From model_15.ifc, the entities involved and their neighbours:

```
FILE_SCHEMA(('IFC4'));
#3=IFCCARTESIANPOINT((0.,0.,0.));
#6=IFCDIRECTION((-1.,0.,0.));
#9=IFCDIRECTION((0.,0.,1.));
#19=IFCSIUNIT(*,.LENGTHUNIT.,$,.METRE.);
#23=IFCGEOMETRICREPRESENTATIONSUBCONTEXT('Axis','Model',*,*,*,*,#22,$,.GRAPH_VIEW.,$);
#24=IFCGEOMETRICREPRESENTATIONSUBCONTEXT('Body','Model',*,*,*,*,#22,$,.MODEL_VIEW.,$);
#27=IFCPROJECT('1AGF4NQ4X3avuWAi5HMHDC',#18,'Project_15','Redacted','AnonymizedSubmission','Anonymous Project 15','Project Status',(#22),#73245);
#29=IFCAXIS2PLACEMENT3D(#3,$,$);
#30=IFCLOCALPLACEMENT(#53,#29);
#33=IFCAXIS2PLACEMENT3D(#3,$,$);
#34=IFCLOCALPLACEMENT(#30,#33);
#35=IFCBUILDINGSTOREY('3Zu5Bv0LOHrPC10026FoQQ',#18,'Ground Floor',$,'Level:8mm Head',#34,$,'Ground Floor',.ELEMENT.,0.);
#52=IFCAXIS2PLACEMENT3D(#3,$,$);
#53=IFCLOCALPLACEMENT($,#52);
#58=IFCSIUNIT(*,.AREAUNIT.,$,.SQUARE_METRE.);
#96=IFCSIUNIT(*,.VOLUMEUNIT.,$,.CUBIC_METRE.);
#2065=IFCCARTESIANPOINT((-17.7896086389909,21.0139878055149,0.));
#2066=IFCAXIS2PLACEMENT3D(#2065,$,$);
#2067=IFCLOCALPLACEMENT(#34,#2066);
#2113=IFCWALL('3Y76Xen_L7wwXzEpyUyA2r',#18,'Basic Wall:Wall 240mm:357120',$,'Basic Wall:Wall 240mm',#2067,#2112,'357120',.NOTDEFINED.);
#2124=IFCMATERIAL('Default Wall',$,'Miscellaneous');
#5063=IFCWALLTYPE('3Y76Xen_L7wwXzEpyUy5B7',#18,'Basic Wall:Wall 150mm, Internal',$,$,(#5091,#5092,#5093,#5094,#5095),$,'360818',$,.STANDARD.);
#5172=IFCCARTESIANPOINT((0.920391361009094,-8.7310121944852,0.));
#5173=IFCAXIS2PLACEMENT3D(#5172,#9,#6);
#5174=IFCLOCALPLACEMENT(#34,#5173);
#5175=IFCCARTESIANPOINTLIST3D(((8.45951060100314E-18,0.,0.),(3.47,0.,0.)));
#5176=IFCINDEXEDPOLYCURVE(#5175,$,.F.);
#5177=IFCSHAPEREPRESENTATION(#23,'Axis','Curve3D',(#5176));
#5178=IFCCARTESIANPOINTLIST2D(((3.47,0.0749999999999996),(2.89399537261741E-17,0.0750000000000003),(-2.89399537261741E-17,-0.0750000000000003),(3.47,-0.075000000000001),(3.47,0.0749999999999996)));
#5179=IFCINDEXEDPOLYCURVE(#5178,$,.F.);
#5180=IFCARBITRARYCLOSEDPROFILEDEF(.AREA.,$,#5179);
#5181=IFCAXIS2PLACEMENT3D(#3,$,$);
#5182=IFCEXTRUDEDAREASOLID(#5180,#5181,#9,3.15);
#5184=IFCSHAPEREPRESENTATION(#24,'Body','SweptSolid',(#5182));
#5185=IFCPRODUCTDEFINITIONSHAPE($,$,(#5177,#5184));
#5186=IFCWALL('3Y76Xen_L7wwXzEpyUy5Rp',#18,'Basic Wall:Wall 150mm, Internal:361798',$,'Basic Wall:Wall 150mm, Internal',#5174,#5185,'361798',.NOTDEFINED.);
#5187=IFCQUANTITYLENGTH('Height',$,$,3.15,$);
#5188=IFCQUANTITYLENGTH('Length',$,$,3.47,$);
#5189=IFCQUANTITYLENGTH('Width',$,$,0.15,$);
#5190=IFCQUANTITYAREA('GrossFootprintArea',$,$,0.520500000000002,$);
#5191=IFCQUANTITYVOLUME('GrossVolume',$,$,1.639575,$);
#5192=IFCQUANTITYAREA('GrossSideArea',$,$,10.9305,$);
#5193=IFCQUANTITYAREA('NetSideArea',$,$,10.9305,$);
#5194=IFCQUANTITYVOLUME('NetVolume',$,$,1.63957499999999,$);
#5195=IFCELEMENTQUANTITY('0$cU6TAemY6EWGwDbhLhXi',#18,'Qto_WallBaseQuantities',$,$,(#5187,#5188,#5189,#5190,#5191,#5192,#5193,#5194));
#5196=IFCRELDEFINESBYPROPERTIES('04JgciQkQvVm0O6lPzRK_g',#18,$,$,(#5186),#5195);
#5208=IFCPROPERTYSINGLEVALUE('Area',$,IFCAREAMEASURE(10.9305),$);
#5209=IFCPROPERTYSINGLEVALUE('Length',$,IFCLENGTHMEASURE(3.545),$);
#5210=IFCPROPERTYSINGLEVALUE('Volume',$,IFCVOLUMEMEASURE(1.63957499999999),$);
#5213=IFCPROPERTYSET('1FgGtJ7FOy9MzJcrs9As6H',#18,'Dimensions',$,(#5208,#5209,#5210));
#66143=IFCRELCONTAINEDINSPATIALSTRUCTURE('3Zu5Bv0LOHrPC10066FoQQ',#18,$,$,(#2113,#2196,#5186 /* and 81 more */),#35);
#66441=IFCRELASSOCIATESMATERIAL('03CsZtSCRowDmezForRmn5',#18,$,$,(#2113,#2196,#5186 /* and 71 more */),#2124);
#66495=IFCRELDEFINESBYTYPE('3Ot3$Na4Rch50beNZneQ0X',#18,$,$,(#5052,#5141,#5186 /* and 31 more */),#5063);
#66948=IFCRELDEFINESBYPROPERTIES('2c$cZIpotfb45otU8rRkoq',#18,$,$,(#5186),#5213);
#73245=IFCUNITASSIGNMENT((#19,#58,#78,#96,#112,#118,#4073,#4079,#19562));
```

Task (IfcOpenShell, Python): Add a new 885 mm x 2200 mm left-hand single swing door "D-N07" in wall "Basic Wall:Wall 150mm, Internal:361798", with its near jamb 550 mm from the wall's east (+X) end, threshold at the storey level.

```python
import numpy as np
import ifcopenshell
import ifcopenshell.api.feature
import ifcopenshell.api.geometry
import ifcopenshell.api.pset
import ifcopenshell.api.root
import ifcopenshell.api.spatial
import ifcopenshell.geom
import ifcopenshell.util.element
import ifcopenshell.util.placement
import ifcopenshell.util.representation
import ifcopenshell.util.shape
import ifcopenshell.util.unit

model = ifcopenshell.open("model_15.ifc")
unit_scale = ifcopenshell.util.unit.calculate_unit_scale(model)
area_scale = ifcopenshell.util.unit.calculate_unit_scale(model, "AREAUNIT")
volume_scale = ifcopenshell.util.unit.calculate_unit_scale(model, "VOLUMEUNIT")
settings = ifcopenshell.geom.settings()


def volume(element):
    """Net volume in cubic metres, openings subtracted."""
    shape = ifcopenshell.geom.create_shape(settings, element)
    return ifcopenshell.util.shape.get_volume(shape.geometry)


wall = model.by_guid("3Y76Xen_L7wwXzEpyUy5Rp")
storey = ifcopenshell.util.element.get_container(wall, ifc_class="IfcBuildingStorey")
context = ifcopenshell.util.representation.get_context(model, "Model", "Body", "MODEL_VIEW")
before = volume(wall)

width, height, from_end, sill = 0.885, 2.2, 0.55, 0.0  # metres

# The wall runs along its own X axis, and the end named is its -X end.
wall_shape = ifcopenshell.geom.create_shape(settings, wall)
x, y, z = ifcopenshell.util.shape.get_vertices(wall_shape.geometry).T
start = x.min() + from_end
face, thickness = float(y.min()), float(y.max() - y.min())
wall_matrix = ifcopenshell.util.placement.get_local_placement(wall.ObjectPlacement)
level = ifcopenshell.util.placement.get_local_placement(storey.ObjectPlacement)[2, 3]


def in_wall(x, y):
    """Placement at x, y metres in the wall's axes, at sill height."""
    matrix = wall_matrix.copy()
    matrix[:, 3] = wall_matrix @ np.array([x / unit_scale, y / unit_scale, 0.0, 1.0])
    matrix[2, 3] = level + sill / unit_scale
    return matrix


# Opening: a box that overshoots both wall faces by 50 mm.
opening = ifcopenshell.api.root.create_entity(model, ifc_class="IfcOpeningElement", predefined_type="OPENING")
box = ifcopenshell.api.geometry.add_wall_representation(
    model, context=context, length=width, height=height, thickness=thickness + 0.1
)
ifcopenshell.api.geometry.assign_representation(model, product=opening, representation=box)
ifcopenshell.api.geometry.edit_object_placement(model, product=opening, matrix=in_wall(start, face - 0.05), is_si=False)
ifcopenshell.api.feature.add_feature(model, feature=opening, element=wall)

door = ifcopenshell.api.root.create_entity(model, ifc_class="IfcDoor", name="D-N07", predefined_type="DOOR")
door.OverallWidth, door.OverallHeight = width / unit_scale, height / unit_scale
door.OperationType = "SINGLE_SWING_LEFT"
body = ifcopenshell.api.geometry.add_door_representation(
    model,
    context=context,
    overall_width=door.OverallWidth,
    overall_height=door.OverallHeight,
    operation_type="SINGLE_SWING_LEFT",
    lining_properties={"LiningDepth": thickness / unit_scale, "ThresholdDepth": thickness / unit_scale},
)
ifcopenshell.api.geometry.assign_representation(model, product=door, representation=body)
ifcopenshell.api.spatial.assign_container(model, products=[door], relating_structure=storey)
ifcopenshell.api.feature.add_filling(model, opening=opening, element=door)

# The lining spans the wall, so the door starts at the wall face.
ifcopenshell.api.geometry.edit_object_placement(model, product=door, matrix=in_wall(start, face), is_si=False)

after = volume(wall)

# Update the wall's stored quantities.
qto = model.by_id(ifcopenshell.util.element.get_pset(wall, "Qto_WallBaseQuantities", should_inherit=False)["id"])
ifcopenshell.api.pset.edit_qto(model, qto=qto, properties={
    "NetSideArea": after / thickness / area_scale,
    "NetVolume": after / volume_scale,
})
pset = model.by_id(ifcopenshell.util.element.get_pset(wall, "Dimensions", should_inherit=False)["id"])
ifcopenshell.api.pset.edit_pset(model, pset=pset, properties={
    "Area": model.create_entity("IfcAreaMeasure", after / thickness / area_scale),
    "Volume": model.create_entity("IfcVolumeMeasure", after / volume_scale),
})

print(f"wall volume {before:.3f} -> {after:.3f} m3")

model.write("model_15_rev.ifc")
```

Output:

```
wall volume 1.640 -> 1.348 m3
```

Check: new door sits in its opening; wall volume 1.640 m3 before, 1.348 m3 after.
